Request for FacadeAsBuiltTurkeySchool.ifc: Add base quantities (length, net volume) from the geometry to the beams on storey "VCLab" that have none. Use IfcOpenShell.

First a look at what the model holds.

```python
import ifcopenshell
import ifcopenshell.util.element
import ifcopenshell.util.unit

model = ifcopenshell.open("FacadeAsBuiltTurkeySchool.ifc")
print(model.schema)
for unit_type in ("LENGTHUNIT", "AREAUNIT", "VOLUMEUNIT"):
    print(unit_type, ifcopenshell.util.unit.calculate_unit_scale(model, unit_type))
storey = next(s for s in model.by_type("IfcBuildingStorey") if s.Name == "VCLab")
beams = [e for e in ifcopenshell.util.element.get_decomposition(storey) if e.is_a("IfcBeam")]
for e in sorted(beams, key=lambda e: e.id()):
    print(e.id(), e.is_a(), e.Name, list(ifcopenshell.util.element.get_psets(e, qtos_only=True)), sep=" | ")
```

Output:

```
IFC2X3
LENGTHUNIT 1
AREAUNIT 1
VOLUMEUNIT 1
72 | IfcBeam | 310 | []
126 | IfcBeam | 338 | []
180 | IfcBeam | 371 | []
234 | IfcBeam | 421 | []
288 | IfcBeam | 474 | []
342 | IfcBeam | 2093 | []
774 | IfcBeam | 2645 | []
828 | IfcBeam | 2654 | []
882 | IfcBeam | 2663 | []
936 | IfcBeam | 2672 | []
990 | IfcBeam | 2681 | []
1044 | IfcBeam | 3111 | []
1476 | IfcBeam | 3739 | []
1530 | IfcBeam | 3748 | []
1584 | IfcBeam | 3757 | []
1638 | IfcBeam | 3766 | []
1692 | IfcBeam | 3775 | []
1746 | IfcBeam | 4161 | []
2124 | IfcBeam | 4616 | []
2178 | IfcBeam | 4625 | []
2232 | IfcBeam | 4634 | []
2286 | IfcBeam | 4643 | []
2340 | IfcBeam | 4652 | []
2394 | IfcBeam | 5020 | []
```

```python
import ifcopenshell
import ifcopenshell.api.pset
import ifcopenshell.geom
import ifcopenshell.util.element
import ifcopenshell.util.shape
import ifcopenshell.util.unit

model = ifcopenshell.open("FacadeAsBuiltTurkeySchool.ifc")
unit_scale = ifcopenshell.util.unit.calculate_unit_scale(model)
volume_scale = ifcopenshell.util.unit.calculate_unit_scale(model, "VOLUMEUNIT")
settings = ifcopenshell.geom.settings()

storey = next(s for s in model.by_type("IfcBuildingStorey") if s.Name == "VCLab")
beams = [e for e in ifcopenshell.util.element.get_decomposition(storey) if e.is_a("IfcBeam")]

for e in sorted(beams, key=lambda e: e.id()):
    if ifcopenshell.util.element.get_psets(e, qtos_only=True, should_inherit=False):
        continue
    # Geometry comes back in metres, in the element's own axes.
    shape = ifcopenshell.geom.create_shape(settings, e)
    values = {
        "Length": ifcopenshell.util.shape.get_max_xyz(shape.geometry) / unit_scale,
        "NetVolume": ifcopenshell.util.shape.get_volume(shape.geometry) / volume_scale,
    }
    qto = ifcopenshell.api.pset.add_qto(model, product=e, name="BaseQuantities")
    ifcopenshell.api.pset.edit_qto(model, qto=qto, properties=values)
    print(e.id(), {k: round(v, 3) for k, v in values.items()})

model.write("FacadeAsBuiltTurkeySchool_updated.ifc")
```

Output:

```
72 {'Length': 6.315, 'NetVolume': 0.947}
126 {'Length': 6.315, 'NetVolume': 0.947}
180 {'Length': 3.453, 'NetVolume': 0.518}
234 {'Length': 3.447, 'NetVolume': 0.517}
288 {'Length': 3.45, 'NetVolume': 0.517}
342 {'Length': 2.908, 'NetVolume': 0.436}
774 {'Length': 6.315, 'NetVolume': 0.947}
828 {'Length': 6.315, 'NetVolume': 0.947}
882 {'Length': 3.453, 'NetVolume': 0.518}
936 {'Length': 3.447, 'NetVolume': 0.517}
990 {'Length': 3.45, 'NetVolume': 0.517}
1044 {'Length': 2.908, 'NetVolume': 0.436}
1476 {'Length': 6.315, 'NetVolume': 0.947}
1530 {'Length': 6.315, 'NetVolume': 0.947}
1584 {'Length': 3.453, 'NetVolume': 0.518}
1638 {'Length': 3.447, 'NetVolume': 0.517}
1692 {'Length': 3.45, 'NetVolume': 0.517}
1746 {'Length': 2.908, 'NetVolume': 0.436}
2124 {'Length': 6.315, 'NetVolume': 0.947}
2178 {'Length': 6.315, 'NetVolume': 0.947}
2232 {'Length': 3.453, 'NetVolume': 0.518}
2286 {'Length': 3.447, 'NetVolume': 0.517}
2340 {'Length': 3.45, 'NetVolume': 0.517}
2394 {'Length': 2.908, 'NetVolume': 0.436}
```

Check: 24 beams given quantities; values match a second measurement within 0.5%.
